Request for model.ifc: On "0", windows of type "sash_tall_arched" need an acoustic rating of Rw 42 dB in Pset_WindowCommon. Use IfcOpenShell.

First a look at what the model holds.

```python
import ifcopenshell
import ifcopenshell.util.element

model = ifcopenshell.open("model.ifc")
print(model.schema)
storey = next(s for s in model.by_type("IfcBuildingStorey") if s.Name == "0")
windows = [e for e in ifcopenshell.util.element.get_decomposition(storey) if e.is_a("IfcWindow")]
seen = {}
for e in windows:
    element_type = ifcopenshell.util.element.get_type(e)
    key = (element_type.Name if element_type != e and element_type else None, ifcopenshell.util.element.get_pset(e, "Pset_WindowCommon", "AcousticRating"))
    seen[key] = seen.get(key, 0) + 1
for (name, value), count in sorted(seen.items(), key=str):
    print(count, "x", name, "|", value)
```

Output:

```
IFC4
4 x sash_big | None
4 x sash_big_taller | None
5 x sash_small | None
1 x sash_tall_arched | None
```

```python
import ifcopenshell
import ifcopenshell.api.pset
import ifcopenshell.util.element

model = ifcopenshell.open("model.ifc")

storey = next(s for s in model.by_type("IfcBuildingStorey") if s.Name == "0")
windows = [e for e in ifcopenshell.util.element.get_decomposition(storey) if e.is_a("IfcWindow")]

count = 0
for e in windows:
    element_type = ifcopenshell.util.element.get_type(e)
    if element_type in (None, e) or element_type.Name != "sash_tall_arched":
        continue
    # add_pset returns the element's existing set when there is one.
    pset = ifcopenshell.api.pset.add_pset(model, product=e, name="Pset_WindowCommon")
    ifcopenshell.api.pset.edit_pset(model, pset=pset, properties={"AcousticRating": "Rw 42 dB"})
    count += 1

print(count, "windows updated")

model.write("model_rev.ifc")
```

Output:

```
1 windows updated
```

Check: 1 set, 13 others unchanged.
